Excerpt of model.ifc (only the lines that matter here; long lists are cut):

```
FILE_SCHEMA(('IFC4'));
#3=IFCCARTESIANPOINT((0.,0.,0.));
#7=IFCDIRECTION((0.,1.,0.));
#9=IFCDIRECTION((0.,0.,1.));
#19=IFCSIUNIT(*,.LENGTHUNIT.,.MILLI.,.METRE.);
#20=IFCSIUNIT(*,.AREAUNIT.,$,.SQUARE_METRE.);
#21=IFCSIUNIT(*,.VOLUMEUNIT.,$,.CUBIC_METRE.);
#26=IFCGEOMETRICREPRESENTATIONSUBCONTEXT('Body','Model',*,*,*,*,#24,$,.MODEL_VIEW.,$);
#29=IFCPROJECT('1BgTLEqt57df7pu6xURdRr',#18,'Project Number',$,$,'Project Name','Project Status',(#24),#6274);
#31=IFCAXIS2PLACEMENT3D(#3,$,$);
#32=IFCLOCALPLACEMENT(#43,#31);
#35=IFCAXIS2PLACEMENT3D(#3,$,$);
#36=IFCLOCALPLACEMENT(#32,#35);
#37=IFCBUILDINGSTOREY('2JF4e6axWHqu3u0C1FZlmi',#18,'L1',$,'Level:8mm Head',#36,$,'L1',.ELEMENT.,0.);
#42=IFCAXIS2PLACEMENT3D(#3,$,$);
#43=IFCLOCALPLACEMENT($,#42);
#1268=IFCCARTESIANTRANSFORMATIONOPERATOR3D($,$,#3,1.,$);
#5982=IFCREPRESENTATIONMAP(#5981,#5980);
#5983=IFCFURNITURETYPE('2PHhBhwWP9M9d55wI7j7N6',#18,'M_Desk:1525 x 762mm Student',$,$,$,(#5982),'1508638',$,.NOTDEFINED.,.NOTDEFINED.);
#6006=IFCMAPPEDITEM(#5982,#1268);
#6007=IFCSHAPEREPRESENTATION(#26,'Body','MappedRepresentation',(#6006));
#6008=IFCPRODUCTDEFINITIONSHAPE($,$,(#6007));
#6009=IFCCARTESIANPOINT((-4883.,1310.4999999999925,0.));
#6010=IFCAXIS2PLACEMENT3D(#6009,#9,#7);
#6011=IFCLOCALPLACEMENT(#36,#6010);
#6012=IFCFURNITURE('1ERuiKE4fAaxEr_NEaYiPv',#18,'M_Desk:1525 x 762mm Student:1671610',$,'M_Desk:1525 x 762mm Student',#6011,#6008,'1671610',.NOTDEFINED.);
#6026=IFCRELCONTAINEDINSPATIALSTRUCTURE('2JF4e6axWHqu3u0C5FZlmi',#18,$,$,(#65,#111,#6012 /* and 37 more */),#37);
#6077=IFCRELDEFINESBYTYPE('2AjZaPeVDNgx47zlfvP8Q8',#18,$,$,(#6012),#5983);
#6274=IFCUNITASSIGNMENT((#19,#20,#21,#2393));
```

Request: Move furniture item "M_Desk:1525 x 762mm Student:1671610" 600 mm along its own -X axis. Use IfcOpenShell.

```python
import ifcopenshell
import ifcopenshell.api.geometry
import ifcopenshell.util.placement

model = ifcopenshell.open("model.ifc")

item = model.by_guid("1ERuiKE4fAaxEr_NEaYiPv")
matrix = ifcopenshell.util.placement.get_local_placement(item.ObjectPlacement)
matrix[:3, 3] -= matrix[:3, 0] * 600.0
ifcopenshell.api.geometry.edit_object_placement(model, product=item, matrix=matrix, is_si=False)

print(ifcopenshell.util.placement.get_local_placement(item.ObjectPlacement).round(3) + 0.0)

model.write("model_updated.ifc")
```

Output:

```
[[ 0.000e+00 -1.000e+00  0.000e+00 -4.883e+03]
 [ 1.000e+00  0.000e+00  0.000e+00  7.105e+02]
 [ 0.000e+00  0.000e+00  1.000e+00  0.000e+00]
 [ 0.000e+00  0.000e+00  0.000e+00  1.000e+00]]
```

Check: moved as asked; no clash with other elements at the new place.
